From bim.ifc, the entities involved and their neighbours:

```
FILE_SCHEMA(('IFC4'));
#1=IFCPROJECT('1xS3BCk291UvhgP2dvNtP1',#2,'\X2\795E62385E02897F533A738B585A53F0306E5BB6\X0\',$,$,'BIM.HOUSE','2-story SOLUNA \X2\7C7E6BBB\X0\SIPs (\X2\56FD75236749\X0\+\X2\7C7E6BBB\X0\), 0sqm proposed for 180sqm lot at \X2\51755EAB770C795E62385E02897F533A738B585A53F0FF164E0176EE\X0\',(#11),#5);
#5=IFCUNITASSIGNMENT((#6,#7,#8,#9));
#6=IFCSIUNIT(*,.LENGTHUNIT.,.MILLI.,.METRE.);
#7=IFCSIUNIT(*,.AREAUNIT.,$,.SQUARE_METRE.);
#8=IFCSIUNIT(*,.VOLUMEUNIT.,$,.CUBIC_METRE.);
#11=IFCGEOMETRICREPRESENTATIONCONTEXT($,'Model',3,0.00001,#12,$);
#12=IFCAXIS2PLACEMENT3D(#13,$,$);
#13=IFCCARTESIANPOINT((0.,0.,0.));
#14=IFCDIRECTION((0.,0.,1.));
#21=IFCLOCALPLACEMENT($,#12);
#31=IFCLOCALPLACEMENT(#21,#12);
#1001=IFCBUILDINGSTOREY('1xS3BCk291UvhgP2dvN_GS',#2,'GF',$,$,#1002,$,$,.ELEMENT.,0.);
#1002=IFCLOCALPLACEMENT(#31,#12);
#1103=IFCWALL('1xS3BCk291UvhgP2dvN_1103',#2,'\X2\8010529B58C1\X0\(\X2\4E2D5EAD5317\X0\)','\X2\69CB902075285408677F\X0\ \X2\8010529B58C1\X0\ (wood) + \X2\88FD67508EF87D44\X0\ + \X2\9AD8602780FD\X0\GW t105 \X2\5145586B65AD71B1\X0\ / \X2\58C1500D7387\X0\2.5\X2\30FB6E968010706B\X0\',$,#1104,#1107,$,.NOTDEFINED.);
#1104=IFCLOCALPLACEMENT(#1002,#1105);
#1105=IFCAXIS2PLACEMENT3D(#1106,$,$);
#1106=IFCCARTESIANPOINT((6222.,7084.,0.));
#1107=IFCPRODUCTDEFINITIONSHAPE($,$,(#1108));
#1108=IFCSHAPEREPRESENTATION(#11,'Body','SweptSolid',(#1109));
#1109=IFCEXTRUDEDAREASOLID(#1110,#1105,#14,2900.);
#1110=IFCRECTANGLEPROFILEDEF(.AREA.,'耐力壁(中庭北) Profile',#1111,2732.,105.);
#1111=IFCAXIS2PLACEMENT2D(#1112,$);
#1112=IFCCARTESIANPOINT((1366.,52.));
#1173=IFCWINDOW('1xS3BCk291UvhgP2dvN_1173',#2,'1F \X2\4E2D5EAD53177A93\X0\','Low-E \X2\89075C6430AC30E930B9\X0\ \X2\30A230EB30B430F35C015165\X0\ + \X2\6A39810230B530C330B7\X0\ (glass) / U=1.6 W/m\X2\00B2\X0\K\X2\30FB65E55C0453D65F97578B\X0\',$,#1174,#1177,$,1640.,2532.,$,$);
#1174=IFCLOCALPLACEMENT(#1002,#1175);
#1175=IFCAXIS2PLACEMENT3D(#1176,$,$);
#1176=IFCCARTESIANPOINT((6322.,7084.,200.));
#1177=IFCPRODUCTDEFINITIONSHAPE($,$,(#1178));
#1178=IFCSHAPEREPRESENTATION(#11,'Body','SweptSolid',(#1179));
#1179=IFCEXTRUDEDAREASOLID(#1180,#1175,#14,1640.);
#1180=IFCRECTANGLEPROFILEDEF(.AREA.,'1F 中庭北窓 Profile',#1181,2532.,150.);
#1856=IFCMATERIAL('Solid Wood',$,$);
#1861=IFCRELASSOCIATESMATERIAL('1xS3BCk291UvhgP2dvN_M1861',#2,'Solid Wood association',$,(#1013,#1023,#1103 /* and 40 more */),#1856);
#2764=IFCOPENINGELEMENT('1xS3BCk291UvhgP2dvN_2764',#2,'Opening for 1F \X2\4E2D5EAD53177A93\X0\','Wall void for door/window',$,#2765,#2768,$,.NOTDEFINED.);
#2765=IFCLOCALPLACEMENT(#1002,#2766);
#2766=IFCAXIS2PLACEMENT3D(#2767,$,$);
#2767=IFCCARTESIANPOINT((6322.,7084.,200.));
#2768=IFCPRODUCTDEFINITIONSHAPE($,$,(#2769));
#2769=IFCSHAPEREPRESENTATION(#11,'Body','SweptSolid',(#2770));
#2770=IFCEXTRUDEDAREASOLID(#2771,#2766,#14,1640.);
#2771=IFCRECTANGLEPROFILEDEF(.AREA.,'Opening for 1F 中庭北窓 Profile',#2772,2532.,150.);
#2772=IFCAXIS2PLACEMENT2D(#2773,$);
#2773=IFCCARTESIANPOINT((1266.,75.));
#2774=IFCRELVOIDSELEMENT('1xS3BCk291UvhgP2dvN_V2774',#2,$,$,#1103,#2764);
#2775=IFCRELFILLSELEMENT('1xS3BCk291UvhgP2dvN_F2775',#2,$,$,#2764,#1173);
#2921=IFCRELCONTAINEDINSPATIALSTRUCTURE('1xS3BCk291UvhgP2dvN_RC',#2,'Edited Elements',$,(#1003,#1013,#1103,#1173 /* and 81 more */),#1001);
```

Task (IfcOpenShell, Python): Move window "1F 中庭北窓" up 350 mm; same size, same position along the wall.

```python
import numpy as np
import ifcopenshell
import ifcopenshell.api.geometry
import ifcopenshell.util.placement
import ifcopenshell.util.unit

model = ifcopenshell.open("bim.ifc")
unit_scale = ifcopenshell.util.unit.calculate_unit_scale(model)

window = model.by_guid("1xS3BCk291UvhgP2dvN_1173")
opening = window.FillsVoids[0].RelatingOpeningElement
dz = 0.35 / unit_scale

shift = np.array([0.0, 0.0, dz])
# The window is not placed relative to its opening, so move both.
for product in (opening, window):
    matrix = ifcopenshell.util.placement.get_local_placement(product.ObjectPlacement)
    matrix[:3, 3] += shift
    ifcopenshell.api.geometry.edit_object_placement(model, product=product, matrix=matrix, is_si=False)

print(f"moved by {dz * unit_scale:+.3f} m")

model.write("bim_edited.ifc")
```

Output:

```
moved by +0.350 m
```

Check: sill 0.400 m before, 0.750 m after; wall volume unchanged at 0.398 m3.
